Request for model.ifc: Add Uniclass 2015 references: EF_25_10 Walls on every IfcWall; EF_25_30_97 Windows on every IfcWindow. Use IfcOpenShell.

First a look at what the model holds.

```python
import ifcopenshell

model = ifcopenshell.open("model.ifc")
print(model.schema)
print("classifications:", [c.Name for c in model.by_type("IfcClassification")])
for ifc_class in ("IfcDoor", "IfcRoof", "IfcStair", "IfcWall", "IfcWindow"):
    print(ifc_class, len(model.by_type(ifc_class)))
```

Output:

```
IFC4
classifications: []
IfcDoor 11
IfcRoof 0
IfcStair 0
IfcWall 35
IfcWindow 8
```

```python
import ifcopenshell
import ifcopenshell.api.classification

model = ifcopenshell.open("model.ifc")

system = ifcopenshell.api.classification.add_classification(model, classification="Uniclass 2015")

codes = {
    "IfcWall": ("EF_25_10", "Walls"),
    "IfcWindow": ("EF_25_30_97", "Windows"),
}
for ifc_class, (code, name) in codes.items():
    products = model.by_type(ifc_class)
    ifcopenshell.api.classification.add_reference(
        model, products=products, classification=system, identification=code, name=name
    )
    print(code, len(products))

model.write("model_rev.ifc")
```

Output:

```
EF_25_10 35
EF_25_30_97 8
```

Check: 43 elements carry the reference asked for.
